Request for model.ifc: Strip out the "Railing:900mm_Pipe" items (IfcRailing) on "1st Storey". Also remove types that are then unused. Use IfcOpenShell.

First a look at what the model holds.

```python
import ifcopenshell
import ifcopenshell.util.element

model = ifcopenshell.open("model.ifc")
print(model.schema)
storey = next(s for s in model.by_type("IfcBuildingStorey") if s.Name == "1st Storey")
railings = [e for e in ifcopenshell.util.element.get_decomposition(storey) if e.is_a("IfcRailing")]
seen = {}
for e in railings:
    element_type = ifcopenshell.util.element.get_type(e)
    name = element_type.Name if element_type not in (None, e) else None
    seen[name] = seen.get(name, 0) + 1
for name, count in sorted(seen.items(), key=str):
    print(count, "x", name)
```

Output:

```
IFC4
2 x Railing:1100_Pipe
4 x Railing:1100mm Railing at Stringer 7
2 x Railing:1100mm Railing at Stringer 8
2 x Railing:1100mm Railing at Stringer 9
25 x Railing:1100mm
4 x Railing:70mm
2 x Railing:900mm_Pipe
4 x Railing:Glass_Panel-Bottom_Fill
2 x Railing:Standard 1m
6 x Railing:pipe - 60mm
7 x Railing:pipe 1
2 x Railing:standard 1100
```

```python
import ifcopenshell
import ifcopenshell.api.root
import ifcopenshell.util.element

model = ifcopenshell.open("model.ifc")

storey = next(s for s in model.by_type("IfcBuildingStorey") if s.Name == "1st Storey")
railings = [e for e in ifcopenshell.util.element.get_decomposition(storey) if e.is_a("IfcRailing")]
targets = [e for e in railings if (t := ifcopenshell.util.element.get_type(e)) not in (None, e) and t.Name == "Railing:900mm_Pipe"]
types = {ifcopenshell.util.element.get_type(e) for e in targets} - {None, *targets}

for e in targets:
    ifcopenshell.api.root.remove_product(model, product=e)
print(len(targets), "removed")

unused = [t for t in types if not ifcopenshell.util.element.get_types(t)]
for t in unused:
    ifcopenshell.api.root.remove_product(model, product=t)
print(len(unused), "unused types removed")

model.write("model_updated.ifc")
```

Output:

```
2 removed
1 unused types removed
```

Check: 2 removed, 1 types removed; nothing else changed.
